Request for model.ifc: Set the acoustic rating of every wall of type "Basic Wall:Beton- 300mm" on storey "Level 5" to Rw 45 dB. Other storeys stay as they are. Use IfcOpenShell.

First a look at what the model holds.

```python
import ifcopenshell
import ifcopenshell.util.element

model = ifcopenshell.open("model.ifc")
print(model.schema)
storey = next(s for s in model.by_type("IfcBuildingStorey") if s.Name == "Level 5")
walls = [e for e in ifcopenshell.util.element.get_decomposition(storey) if e.is_a("IfcWall")]
seen = {}
for e in walls:
    element_type = ifcopenshell.util.element.get_type(e)
    key = (element_type.Name if element_type != e and element_type else None, ifcopenshell.util.element.get_pset(e, "Pset_WallCommon", "AcousticRating"))
    seen[key] = seen.get(key, 0) + 1
for (name, value), count in sorted(seen.items(), key=str):
    print(count, "x", name, "|", value)
```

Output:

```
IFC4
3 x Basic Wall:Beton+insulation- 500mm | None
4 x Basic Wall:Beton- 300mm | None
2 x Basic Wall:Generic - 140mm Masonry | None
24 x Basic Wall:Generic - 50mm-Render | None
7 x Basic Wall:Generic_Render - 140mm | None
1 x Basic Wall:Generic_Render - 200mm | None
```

```python
import ifcopenshell
import ifcopenshell.api.pset
import ifcopenshell.util.element

model = ifcopenshell.open("model.ifc")

storey = next(s for s in model.by_type("IfcBuildingStorey") if s.Name == "Level 5")
walls = [e for e in ifcopenshell.util.element.get_decomposition(storey) if e.is_a("IfcWall")]

count = 0
for e in walls:
    element_type = ifcopenshell.util.element.get_type(e)
    if element_type in (None, e) or element_type.Name != "Basic Wall:Beton- 300mm":
        continue
    # add_pset returns the element's existing set when there is one.
    pset = ifcopenshell.api.pset.add_pset(model, product=e, name="Pset_WallCommon")
    ifcopenshell.api.pset.edit_pset(model, pset=pset, properties={"AcousticRating": "Rw 45 dB"})
    count += 1

print(count, "walls updated")

model.write("model_edited.ifc")
```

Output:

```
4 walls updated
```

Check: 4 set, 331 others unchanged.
